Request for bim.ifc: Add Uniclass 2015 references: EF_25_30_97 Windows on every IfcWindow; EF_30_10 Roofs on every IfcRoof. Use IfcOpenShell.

First a look at what the model holds.

```python
import ifcopenshell

model = ifcopenshell.open("bim.ifc")
print(model.schema)
print("classifications:", [c.Name for c in model.by_type("IfcClassification")])
for ifc_class in ("IfcDoor", "IfcRoof", "IfcStair", "IfcWall", "IfcWindow"):
    print(ifc_class, len(model.by_type(ifc_class)))
```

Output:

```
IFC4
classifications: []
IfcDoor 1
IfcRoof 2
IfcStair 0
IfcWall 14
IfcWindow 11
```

```python
import ifcopenshell
import ifcopenshell.api.classification

model = ifcopenshell.open("bim.ifc")

system = ifcopenshell.api.classification.add_classification(model, classification="Uniclass 2015")

codes = {
    "IfcWindow": ("EF_25_30_97", "Windows"),
    "IfcRoof": ("EF_30_10", "Roofs"),
}
for ifc_class, (code, name) in codes.items():
    products = model.by_type(ifc_class)
    ifcopenshell.api.classification.add_reference(
        model, products=products, classification=system, identification=code, name=name
    )
    print(code, len(products))

model.write("bim_rev.ifc")
```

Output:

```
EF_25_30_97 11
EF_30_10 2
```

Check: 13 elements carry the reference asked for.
